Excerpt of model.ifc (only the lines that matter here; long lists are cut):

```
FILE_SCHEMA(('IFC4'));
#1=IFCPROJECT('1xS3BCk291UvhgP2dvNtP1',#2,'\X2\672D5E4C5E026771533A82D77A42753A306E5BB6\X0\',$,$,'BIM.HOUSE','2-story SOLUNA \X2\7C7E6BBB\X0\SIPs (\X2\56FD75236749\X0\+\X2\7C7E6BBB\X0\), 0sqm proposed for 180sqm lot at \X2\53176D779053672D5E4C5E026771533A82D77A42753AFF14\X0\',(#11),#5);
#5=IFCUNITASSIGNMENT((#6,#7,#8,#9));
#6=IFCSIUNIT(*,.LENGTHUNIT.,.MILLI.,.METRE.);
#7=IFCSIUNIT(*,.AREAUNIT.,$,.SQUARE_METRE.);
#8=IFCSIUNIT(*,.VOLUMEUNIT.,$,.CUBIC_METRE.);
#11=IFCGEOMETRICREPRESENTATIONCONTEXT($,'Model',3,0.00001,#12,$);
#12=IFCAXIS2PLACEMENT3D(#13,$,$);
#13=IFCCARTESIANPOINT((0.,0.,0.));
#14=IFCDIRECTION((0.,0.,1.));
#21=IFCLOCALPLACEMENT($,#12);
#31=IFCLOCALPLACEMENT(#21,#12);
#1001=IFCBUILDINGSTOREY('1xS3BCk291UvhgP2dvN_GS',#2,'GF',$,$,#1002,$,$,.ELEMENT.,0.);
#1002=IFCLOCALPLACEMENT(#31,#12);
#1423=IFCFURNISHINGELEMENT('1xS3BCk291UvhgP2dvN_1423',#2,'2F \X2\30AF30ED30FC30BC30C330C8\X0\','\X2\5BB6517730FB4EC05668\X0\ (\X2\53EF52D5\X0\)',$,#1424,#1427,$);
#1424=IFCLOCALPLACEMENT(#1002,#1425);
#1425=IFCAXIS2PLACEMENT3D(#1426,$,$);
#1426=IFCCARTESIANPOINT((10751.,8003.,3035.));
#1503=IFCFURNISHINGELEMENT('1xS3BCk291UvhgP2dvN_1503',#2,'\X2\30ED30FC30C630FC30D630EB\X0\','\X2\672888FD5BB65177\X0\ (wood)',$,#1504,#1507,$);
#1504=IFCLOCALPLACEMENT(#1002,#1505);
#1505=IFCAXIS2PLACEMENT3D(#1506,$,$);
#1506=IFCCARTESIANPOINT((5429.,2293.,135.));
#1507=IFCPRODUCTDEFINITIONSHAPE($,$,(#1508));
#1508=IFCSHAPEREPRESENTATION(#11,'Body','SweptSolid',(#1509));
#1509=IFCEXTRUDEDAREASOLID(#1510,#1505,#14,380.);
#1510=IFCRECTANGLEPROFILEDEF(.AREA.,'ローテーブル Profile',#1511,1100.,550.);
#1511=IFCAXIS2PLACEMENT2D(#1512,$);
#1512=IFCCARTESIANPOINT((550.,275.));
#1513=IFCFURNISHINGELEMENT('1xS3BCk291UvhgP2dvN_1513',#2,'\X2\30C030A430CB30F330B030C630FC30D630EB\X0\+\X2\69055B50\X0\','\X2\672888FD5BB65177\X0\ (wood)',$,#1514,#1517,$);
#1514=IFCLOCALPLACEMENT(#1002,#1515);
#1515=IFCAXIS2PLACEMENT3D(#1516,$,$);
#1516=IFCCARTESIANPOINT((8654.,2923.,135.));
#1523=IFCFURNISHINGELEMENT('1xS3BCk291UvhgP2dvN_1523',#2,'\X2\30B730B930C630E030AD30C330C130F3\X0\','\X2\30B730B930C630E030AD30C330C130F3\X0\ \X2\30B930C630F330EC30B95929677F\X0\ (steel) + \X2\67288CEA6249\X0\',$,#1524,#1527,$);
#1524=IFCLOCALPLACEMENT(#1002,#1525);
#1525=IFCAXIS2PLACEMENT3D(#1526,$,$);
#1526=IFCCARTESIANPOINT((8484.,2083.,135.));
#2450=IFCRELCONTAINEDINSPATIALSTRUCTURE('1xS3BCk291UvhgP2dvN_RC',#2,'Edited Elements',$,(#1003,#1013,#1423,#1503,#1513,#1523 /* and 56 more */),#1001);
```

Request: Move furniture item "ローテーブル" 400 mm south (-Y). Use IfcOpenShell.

```python
import ifcopenshell
import ifcopenshell.api.geometry
import ifcopenshell.util.placement

model = ifcopenshell.open("model.ifc")

item = model.by_guid("1xS3BCk291UvhgP2dvN_1503")
matrix = ifcopenshell.util.placement.get_local_placement(item.ObjectPlacement)
matrix[1, 3] -= 400.0
ifcopenshell.api.geometry.edit_object_placement(model, product=item, matrix=matrix, is_si=False)

print(ifcopenshell.util.placement.get_local_placement(item.ObjectPlacement).round(3) + 0.0)

model.write("model_edited.ifc")
```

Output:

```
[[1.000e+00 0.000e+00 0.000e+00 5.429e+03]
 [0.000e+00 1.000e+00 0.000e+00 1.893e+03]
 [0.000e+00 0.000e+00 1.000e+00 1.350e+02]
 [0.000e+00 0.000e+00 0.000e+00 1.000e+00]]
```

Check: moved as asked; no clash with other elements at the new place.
